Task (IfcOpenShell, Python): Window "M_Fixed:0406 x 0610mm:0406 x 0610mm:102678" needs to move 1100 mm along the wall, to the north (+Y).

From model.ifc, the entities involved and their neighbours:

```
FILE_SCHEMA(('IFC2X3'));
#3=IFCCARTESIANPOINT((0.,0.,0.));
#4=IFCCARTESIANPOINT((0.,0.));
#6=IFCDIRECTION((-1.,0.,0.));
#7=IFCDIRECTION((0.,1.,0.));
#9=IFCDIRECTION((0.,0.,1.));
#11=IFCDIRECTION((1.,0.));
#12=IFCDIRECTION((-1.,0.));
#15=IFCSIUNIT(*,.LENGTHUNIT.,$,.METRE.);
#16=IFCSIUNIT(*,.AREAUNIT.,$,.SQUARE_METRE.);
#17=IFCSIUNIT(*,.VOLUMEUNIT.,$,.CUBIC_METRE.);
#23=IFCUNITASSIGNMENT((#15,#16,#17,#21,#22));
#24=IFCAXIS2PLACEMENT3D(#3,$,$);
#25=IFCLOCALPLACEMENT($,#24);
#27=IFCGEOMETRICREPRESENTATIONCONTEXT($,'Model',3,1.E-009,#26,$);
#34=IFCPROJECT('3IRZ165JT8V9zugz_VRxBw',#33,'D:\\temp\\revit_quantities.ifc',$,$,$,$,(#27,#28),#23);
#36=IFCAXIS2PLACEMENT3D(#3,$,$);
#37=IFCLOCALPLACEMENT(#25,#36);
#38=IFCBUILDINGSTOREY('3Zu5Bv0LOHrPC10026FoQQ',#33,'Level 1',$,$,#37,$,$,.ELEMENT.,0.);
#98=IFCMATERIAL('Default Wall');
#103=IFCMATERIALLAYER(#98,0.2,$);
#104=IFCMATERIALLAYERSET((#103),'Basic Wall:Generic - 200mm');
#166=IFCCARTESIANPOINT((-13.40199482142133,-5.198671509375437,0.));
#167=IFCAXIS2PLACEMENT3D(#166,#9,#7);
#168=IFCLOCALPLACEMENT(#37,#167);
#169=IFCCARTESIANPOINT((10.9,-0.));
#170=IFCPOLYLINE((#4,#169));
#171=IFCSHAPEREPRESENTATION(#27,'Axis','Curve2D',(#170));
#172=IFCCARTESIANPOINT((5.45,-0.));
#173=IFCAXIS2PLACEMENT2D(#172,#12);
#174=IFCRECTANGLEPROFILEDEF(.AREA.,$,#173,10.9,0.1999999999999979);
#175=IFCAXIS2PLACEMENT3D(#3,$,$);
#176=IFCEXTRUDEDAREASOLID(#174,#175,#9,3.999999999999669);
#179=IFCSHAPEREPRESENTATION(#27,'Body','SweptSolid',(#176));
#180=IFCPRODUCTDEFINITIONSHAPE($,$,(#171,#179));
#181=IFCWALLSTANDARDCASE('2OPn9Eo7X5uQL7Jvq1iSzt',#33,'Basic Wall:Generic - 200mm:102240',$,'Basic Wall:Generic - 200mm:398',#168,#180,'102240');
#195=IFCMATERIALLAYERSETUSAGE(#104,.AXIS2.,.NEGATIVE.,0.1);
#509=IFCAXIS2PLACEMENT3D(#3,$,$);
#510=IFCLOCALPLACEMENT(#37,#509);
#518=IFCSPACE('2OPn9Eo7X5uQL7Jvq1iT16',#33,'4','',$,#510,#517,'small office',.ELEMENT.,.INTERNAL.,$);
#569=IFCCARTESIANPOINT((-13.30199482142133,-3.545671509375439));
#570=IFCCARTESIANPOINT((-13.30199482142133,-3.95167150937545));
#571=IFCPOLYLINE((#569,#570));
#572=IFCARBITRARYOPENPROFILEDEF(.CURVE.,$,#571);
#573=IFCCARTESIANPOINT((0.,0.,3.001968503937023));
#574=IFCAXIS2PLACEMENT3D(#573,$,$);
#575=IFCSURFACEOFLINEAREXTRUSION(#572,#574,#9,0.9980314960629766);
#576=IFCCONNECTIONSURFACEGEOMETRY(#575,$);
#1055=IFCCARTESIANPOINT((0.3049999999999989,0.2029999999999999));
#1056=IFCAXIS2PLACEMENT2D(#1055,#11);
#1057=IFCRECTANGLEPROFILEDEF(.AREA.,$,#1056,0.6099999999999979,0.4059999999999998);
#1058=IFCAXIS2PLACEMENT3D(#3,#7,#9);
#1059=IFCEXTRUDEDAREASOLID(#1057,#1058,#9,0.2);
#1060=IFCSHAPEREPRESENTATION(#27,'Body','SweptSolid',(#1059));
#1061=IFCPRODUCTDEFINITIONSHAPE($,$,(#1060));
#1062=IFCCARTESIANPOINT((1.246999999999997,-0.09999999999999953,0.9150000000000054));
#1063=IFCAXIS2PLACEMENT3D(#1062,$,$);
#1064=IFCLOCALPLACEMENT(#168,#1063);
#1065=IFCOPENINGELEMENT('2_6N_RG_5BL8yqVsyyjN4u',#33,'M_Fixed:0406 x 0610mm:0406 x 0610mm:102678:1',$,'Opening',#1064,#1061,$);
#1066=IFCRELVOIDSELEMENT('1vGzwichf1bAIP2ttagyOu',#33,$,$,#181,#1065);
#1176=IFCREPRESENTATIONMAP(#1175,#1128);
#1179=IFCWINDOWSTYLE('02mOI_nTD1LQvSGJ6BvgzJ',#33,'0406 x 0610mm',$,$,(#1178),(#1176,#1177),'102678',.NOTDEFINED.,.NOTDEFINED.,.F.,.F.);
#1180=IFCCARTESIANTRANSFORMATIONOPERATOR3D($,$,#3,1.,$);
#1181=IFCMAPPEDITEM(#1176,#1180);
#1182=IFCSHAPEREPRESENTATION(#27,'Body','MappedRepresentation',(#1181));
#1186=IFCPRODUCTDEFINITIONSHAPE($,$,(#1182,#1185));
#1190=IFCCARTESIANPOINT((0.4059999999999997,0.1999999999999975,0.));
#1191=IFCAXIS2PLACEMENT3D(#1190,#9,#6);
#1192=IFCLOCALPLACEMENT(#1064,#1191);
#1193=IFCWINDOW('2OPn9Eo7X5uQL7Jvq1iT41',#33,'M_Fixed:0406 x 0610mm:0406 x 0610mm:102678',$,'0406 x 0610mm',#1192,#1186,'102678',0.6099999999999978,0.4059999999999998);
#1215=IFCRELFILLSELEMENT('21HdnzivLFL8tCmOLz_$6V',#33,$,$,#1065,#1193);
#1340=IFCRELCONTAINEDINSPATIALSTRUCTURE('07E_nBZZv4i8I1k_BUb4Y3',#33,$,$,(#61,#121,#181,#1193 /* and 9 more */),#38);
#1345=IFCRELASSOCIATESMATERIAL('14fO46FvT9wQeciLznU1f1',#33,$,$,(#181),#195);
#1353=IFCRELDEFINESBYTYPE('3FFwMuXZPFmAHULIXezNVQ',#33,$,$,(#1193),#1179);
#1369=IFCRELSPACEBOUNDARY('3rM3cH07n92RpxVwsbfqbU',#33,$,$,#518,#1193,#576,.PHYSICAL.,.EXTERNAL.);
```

```python
import numpy as np
import ifcopenshell
import ifcopenshell.api.geometry
import ifcopenshell.util.placement

model = ifcopenshell.open("model.ifc")

window = model.by_guid("2OPn9Eo7X5uQL7Jvq1iT41")
opening = window.FillsVoids[0].RelatingOpeningElement
wall = opening.VoidsElements[0].RelatingBuildingElement

wall_matrix = ifcopenshell.util.placement.get_local_placement(wall.ObjectPlacement)
shift = wall_matrix[:3, 0] * 1.1
before = ifcopenshell.util.placement.get_local_placement(window.ObjectPlacement)[:3, 3].copy()

# The window is placed relative to its opening, so it follows when the opening moves.
matrix = ifcopenshell.util.placement.get_local_placement(opening.ObjectPlacement)
matrix[:3, 3] += shift
ifcopenshell.api.geometry.edit_object_placement(
    model, product=opening, matrix=matrix, is_si=False, should_transform_children=True
)

# Space boundary surfaces are stored in each space's coordinates; move them too.
for rel in window.ProvidesBoundaries:
    if not rel.ConnectionGeometry:
        continue
    surface = rel.ConnectionGeometry.SurfaceOnRelatingElement
    space_matrix = ifcopenshell.util.placement.get_local_placement(rel.RelatingSpace.ObjectPlacement)
    point = np.array(surface.Position.Location.Coordinates) + space_matrix[:3, :3].T @ shift
    surface.Position = model.createIfcAxis2Placement3D(
        model.createIfcCartesianPoint(point.tolist()), surface.Position.Axis, surface.Position.RefDirection
    )

after = ifcopenshell.util.placement.get_local_placement(window.ObjectPlacement)[:3, 3]
print("window moved by", (after - before).round(3) + 0.0)

model.write("model_rev.ifc")
```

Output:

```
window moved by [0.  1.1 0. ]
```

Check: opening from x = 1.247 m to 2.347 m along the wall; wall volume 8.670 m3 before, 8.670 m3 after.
